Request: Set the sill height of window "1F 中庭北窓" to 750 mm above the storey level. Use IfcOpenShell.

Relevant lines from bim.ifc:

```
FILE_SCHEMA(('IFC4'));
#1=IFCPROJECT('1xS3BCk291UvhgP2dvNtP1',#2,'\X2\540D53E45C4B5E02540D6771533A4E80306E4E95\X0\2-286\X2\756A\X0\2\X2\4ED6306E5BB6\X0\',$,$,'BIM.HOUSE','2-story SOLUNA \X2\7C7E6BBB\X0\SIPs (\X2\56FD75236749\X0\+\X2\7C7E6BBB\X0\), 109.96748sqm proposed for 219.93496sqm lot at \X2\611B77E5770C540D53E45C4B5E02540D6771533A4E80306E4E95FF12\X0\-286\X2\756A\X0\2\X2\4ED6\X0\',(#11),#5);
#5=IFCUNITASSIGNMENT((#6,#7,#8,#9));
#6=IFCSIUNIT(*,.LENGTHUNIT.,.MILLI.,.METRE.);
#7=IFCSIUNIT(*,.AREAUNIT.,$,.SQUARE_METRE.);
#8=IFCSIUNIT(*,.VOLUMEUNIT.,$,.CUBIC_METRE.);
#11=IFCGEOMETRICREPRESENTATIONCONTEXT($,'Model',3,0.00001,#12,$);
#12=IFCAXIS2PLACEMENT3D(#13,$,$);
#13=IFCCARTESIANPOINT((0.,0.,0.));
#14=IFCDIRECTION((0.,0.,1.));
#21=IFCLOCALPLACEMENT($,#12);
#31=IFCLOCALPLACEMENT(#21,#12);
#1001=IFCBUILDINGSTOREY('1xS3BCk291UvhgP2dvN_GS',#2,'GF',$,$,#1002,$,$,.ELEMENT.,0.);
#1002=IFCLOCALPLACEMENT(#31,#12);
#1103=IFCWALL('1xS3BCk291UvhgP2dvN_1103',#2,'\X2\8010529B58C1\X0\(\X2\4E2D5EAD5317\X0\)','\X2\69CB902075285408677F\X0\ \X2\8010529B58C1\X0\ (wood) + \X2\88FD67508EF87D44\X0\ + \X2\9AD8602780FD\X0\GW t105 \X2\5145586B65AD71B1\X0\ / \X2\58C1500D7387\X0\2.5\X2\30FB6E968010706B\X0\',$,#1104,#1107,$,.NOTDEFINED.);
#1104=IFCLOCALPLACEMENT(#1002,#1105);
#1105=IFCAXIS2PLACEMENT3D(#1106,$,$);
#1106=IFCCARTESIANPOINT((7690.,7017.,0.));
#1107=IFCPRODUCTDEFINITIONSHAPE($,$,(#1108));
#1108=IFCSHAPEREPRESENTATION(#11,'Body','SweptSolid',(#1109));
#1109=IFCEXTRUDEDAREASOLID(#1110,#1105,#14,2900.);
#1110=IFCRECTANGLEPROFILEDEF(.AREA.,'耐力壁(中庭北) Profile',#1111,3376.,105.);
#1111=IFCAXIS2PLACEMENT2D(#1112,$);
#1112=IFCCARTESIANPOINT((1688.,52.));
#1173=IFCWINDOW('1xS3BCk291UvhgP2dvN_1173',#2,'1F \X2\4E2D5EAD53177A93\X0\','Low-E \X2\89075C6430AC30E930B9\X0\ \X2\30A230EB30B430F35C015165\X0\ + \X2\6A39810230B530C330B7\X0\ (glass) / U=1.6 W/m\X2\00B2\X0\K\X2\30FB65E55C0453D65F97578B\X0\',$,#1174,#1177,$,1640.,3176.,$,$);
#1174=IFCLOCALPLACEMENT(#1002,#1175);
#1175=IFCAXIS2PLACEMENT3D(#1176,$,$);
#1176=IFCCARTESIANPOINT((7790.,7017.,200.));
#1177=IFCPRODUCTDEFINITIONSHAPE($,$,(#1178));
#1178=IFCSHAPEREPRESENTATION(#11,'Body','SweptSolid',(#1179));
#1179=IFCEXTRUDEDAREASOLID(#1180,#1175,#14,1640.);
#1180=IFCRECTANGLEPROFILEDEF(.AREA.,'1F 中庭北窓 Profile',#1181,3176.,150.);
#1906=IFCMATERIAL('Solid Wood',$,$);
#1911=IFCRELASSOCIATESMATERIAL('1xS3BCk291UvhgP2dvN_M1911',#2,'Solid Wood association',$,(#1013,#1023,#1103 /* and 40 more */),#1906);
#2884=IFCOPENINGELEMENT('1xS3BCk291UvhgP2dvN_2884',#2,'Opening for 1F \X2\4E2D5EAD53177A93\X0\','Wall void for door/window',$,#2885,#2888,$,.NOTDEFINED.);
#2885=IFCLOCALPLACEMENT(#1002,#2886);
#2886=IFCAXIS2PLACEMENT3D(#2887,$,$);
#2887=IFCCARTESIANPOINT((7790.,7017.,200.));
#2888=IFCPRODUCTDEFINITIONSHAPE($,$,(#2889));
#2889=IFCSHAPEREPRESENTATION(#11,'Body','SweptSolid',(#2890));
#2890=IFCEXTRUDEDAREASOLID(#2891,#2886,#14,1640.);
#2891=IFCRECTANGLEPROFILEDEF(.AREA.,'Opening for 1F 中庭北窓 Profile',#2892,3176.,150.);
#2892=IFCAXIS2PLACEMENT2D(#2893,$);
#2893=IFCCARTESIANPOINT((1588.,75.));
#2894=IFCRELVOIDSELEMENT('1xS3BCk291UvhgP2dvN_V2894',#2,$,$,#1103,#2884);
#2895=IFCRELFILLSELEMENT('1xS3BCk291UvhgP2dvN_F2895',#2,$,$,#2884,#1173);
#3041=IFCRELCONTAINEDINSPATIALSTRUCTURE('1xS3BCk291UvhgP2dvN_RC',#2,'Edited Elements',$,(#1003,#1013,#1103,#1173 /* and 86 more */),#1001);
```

```python
import numpy as np
import ifcopenshell
import ifcopenshell.api.geometry
import ifcopenshell.geom
import ifcopenshell.util.element
import ifcopenshell.util.placement
import ifcopenshell.util.shape
import ifcopenshell.util.unit

model = ifcopenshell.open("bim.ifc")
unit_scale = ifcopenshell.util.unit.calculate_unit_scale(model)

window = model.by_guid("1xS3BCk291UvhgP2dvN_1173")
opening = window.FillsVoids[0].RelatingOpeningElement
storey = ifcopenshell.util.element.get_container(window, ifc_class="IfcBuildingStorey")
level = ifcopenshell.util.placement.get_local_placement(storey.ObjectPlacement)[2, 3]

# The opening's origin need not be at the sill, so measure its lowest point.
shape = ifcopenshell.geom.create_shape(ifcopenshell.geom.settings(), opening)
bottom = ifcopenshell.util.shape.get_shape_bottom_elevation(shape, shape.geometry) / unit_scale
dz = level + 750.0 - bottom

shift = np.array([0.0, 0.0, dz])
# The window is not placed relative to its opening, so move both.
for product in (opening, window):
    matrix = ifcopenshell.util.placement.get_local_placement(product.ObjectPlacement)
    matrix[:3, 3] += shift
    ifcopenshell.api.geometry.edit_object_placement(model, product=product, matrix=matrix, is_si=False)

print(f"moved by {dz * unit_scale:+.3f} m")

model.write("bim_updated.ifc")
```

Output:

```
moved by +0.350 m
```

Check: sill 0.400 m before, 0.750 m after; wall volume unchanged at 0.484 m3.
